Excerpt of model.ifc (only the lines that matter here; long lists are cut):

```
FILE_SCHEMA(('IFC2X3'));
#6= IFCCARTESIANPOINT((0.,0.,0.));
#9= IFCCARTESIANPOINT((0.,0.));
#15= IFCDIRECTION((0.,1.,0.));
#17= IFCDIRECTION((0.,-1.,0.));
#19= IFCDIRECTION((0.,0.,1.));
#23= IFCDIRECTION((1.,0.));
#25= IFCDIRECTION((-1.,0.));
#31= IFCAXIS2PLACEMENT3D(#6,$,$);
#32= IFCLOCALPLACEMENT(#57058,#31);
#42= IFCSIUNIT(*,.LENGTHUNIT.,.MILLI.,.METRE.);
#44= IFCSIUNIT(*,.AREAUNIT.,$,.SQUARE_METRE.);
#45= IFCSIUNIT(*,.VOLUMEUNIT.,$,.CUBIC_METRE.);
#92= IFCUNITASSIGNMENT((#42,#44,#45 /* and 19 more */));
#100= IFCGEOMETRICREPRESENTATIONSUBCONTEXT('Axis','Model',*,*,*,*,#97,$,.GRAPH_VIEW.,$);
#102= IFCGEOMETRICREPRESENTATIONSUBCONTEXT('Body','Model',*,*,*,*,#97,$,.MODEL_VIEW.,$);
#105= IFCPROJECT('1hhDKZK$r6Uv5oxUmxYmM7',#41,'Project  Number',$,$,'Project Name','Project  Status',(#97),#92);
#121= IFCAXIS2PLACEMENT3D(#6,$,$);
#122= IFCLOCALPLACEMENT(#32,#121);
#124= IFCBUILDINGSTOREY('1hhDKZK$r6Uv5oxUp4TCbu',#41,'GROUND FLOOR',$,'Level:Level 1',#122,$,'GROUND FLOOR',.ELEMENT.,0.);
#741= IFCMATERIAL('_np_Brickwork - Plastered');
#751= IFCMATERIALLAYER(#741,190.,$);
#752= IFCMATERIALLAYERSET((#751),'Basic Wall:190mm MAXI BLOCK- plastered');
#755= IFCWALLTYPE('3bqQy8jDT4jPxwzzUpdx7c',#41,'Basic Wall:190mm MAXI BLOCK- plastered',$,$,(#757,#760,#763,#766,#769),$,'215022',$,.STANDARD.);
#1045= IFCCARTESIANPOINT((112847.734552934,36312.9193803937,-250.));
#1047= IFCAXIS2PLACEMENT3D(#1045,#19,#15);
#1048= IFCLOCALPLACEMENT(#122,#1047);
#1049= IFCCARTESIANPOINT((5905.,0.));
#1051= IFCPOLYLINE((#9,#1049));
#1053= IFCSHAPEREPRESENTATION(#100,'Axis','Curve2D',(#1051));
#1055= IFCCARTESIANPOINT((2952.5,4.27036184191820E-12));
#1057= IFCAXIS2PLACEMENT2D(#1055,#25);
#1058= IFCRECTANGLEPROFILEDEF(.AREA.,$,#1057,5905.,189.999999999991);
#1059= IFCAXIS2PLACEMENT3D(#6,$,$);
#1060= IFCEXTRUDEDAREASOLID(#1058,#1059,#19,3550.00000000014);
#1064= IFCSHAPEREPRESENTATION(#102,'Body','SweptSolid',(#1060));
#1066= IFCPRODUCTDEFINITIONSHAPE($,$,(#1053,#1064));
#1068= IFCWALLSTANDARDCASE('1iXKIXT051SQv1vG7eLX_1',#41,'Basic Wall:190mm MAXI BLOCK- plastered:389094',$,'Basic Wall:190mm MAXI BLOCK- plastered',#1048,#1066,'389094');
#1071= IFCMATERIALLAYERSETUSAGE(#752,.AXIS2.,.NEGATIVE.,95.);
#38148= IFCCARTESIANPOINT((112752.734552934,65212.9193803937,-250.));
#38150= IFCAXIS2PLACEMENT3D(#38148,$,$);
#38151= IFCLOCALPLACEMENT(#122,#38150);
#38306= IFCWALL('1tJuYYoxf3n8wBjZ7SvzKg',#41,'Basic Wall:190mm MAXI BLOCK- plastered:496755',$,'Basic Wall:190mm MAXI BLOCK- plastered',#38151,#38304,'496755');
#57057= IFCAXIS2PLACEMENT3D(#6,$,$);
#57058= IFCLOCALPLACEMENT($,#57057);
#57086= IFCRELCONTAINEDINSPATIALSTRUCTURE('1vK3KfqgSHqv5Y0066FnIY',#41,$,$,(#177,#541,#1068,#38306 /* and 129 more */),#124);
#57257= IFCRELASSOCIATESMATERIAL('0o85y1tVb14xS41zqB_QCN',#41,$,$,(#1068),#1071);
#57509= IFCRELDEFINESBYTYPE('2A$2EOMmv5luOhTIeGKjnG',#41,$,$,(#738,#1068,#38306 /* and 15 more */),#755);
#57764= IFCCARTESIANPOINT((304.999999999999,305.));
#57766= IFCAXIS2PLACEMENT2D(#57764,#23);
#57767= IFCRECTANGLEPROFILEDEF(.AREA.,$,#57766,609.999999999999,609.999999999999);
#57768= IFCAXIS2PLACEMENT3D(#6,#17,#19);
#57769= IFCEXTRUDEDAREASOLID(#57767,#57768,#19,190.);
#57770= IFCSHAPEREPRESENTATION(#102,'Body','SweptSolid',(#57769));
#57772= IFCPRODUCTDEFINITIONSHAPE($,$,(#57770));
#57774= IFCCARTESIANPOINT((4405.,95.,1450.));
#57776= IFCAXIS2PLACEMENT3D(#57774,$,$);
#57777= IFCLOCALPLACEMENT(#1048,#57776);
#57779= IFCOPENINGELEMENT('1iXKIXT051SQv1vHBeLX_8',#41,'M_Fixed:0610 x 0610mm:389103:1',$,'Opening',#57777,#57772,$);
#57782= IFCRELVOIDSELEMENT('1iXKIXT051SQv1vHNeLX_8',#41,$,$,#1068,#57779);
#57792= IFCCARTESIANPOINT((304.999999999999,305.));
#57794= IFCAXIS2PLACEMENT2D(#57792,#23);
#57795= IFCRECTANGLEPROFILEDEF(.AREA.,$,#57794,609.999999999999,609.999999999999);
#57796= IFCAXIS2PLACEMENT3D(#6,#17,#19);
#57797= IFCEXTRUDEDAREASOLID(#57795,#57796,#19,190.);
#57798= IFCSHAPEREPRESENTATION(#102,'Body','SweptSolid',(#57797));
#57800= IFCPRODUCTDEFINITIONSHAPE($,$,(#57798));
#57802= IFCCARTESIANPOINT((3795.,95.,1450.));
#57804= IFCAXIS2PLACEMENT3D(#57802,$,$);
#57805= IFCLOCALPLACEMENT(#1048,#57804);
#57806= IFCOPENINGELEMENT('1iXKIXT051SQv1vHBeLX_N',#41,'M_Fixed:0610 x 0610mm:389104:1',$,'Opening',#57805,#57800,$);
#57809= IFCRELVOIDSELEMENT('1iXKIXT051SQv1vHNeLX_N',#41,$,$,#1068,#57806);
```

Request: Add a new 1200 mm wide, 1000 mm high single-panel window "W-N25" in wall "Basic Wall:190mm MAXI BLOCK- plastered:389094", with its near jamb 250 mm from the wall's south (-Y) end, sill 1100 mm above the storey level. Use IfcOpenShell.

```python
import numpy as np
import ifcopenshell
import ifcopenshell.api.feature
import ifcopenshell.api.geometry
import ifcopenshell.api.root
import ifcopenshell.api.spatial
import ifcopenshell.api.type
import ifcopenshell.geom
import ifcopenshell.util.element
import ifcopenshell.util.placement
import ifcopenshell.util.representation
import ifcopenshell.util.shape
import ifcopenshell.util.unit

model = ifcopenshell.open("model.ifc")
unit_scale = ifcopenshell.util.unit.calculate_unit_scale(model)
settings = ifcopenshell.geom.settings()


def volume(element):
    """Net volume in cubic metres, openings subtracted."""
    shape = ifcopenshell.geom.create_shape(settings, element)
    return ifcopenshell.util.shape.get_volume(shape.geometry)


wall = model.by_guid("1iXKIXT051SQv1vG7eLX_1")
storey = ifcopenshell.util.element.get_container(wall, ifc_class="IfcBuildingStorey")
context = ifcopenshell.util.representation.get_context(model, "Model", "Body", "MODEL_VIEW")
before = volume(wall)

width, height, from_end, sill = 1.2, 1, 0.25, 1.1  # metres

# The wall runs along its own X axis, and the end named is its -X end.
wall_shape = ifcopenshell.geom.create_shape(settings, wall)
x, y, z = ifcopenshell.util.shape.get_vertices(wall_shape.geometry).T
start = x.min() + from_end
face, thickness = float(y.min()), float(y.max() - y.min())
wall_matrix = ifcopenshell.util.placement.get_local_placement(wall.ObjectPlacement)
level = ifcopenshell.util.placement.get_local_placement(storey.ObjectPlacement)[2, 3]


def in_wall(x, y):
    """Placement at x, y metres in the wall's axes, at sill height."""
    matrix = wall_matrix.copy()
    matrix[:, 3] = wall_matrix @ np.array([x / unit_scale, y / unit_scale, 0.0, 1.0])
    matrix[2, 3] = level + sill / unit_scale
    return matrix


# Opening: a box that overshoots both wall faces by 50 mm.
opening = ifcopenshell.api.root.create_entity(model, ifc_class="IfcOpeningElement")
box = ifcopenshell.api.geometry.add_wall_representation(
    model, context=context, length=width, height=height, thickness=thickness + 0.1
)
ifcopenshell.api.geometry.assign_representation(model, product=opening, representation=box)
ifcopenshell.api.geometry.edit_object_placement(model, product=opening, matrix=in_wall(start, face - 0.05), is_si=False)
ifcopenshell.api.feature.add_feature(model, feature=opening, element=wall)

window = ifcopenshell.api.root.create_entity(model, ifc_class="IfcWindow", name="W-N25")
window.OverallWidth, window.OverallHeight = width / unit_scale, height / unit_scale
body = ifcopenshell.api.geometry.add_window_representation(
    model,
    context=context,
    overall_width=window.OverallWidth,
    overall_height=window.OverallHeight,
    partition_type="SINGLE_PANEL",
)
ifcopenshell.api.geometry.assign_representation(model, product=window, representation=body)
ifcopenshell.api.spatial.assign_container(model, products=[window], relating_structure=storey)
fills = ifcopenshell.api.feature.add_filling(model, opening=opening, element=window)
fills.OwnerHistory = window.OwnerHistory  # required in IFC2X3

# IFC2X3 keeps the operation on the window style.
style = ifcopenshell.api.root.create_entity(model, ifc_class="IfcWindowStyle", name="W-N25")
style.OperationType, style.ConstructionType = "SINGLE_PANEL", "NOTDEFINED"
style.ParameterTakesPrecedence = style.Sizeable = False
ifcopenshell.api.type.assign_type(model, related_objects=[window], relating_type=style)

# Centre the window in the wall's thickness.
ifcopenshell.api.geometry.edit_object_placement(model, product=window, matrix=in_wall(start, face), is_si=False)
window_shape = ifcopenshell.geom.create_shape(settings, window)
depth = ifcopenshell.util.shape.get_vertices(window_shape.geometry)[:, 1]
offset = face + thickness / 2 - (depth.min() + depth.max()) / 2
ifcopenshell.api.geometry.edit_object_placement(model, product=window, matrix=in_wall(start, offset), is_si=False)

after = volume(wall)

print(f"wall volume {before:.3f} -> {after:.3f} m3")

model.write("model_edited.ifc")
```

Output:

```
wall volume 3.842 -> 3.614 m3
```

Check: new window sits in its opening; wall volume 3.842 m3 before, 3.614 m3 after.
